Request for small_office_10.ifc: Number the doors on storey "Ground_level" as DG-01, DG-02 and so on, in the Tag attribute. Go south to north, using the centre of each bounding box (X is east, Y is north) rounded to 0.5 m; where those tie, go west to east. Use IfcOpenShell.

First a look at what the model holds.

```python
import ifcopenshell
import ifcopenshell.util.element
import ifcopenshell.util.placement

model = ifcopenshell.open("small_office_10.ifc")
print(model.schema)
storey = next(s for s in model.by_type("IfcBuildingStorey") if s.Name == "Ground_level")
doors = [e for e in ifcopenshell.util.element.get_decomposition(storey) if e.is_a("IfcDoor")]
for e in sorted(doors, key=lambda e: e.id()):
    origin = ifcopenshell.util.placement.get_local_placement(e.ObjectPlacement)[:3, 3]
    print(e.id(), e.Tag, e.Name, origin.round(2) + 0.0, sep=" | ")
```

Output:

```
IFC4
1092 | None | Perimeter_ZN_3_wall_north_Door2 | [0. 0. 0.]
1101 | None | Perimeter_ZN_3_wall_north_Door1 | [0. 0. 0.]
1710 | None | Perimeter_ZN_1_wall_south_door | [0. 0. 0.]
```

```python
import ifcopenshell
import ifcopenshell.geom
import ifcopenshell.util.element
import ifcopenshell.util.shape

model = ifcopenshell.open("small_office_10.ifc")
settings = ifcopenshell.geom.settings()
settings.set("use-world-coords", True)


def centre(element):
    shape = ifcopenshell.geom.create_shape(settings, element)
    return ifcopenshell.util.shape.get_bbox_centroid(shape.geometry)


storey = next(s for s in model.by_type("IfcBuildingStorey") if s.Name == "Ground_level")
doors = [e for e in ifcopenshell.util.element.get_decomposition(storey) if e.is_a("IfcDoor")]

# Insertion points can sit at a corner or the storey origin, so sort by the geometry (in metres).
centres = {e: centre(e) for e in doors}
doors.sort(key=lambda e: (round(centres[e][1] / 0.5), centres[e][0]))

for i, e in enumerate(doors, start=1):
    number = f"DG-{i:02d}"
    e.Tag = number
    print(e.id(), number)

model.write("small_office_10_edited.ifc")
```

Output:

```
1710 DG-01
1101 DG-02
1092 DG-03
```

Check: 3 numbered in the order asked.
